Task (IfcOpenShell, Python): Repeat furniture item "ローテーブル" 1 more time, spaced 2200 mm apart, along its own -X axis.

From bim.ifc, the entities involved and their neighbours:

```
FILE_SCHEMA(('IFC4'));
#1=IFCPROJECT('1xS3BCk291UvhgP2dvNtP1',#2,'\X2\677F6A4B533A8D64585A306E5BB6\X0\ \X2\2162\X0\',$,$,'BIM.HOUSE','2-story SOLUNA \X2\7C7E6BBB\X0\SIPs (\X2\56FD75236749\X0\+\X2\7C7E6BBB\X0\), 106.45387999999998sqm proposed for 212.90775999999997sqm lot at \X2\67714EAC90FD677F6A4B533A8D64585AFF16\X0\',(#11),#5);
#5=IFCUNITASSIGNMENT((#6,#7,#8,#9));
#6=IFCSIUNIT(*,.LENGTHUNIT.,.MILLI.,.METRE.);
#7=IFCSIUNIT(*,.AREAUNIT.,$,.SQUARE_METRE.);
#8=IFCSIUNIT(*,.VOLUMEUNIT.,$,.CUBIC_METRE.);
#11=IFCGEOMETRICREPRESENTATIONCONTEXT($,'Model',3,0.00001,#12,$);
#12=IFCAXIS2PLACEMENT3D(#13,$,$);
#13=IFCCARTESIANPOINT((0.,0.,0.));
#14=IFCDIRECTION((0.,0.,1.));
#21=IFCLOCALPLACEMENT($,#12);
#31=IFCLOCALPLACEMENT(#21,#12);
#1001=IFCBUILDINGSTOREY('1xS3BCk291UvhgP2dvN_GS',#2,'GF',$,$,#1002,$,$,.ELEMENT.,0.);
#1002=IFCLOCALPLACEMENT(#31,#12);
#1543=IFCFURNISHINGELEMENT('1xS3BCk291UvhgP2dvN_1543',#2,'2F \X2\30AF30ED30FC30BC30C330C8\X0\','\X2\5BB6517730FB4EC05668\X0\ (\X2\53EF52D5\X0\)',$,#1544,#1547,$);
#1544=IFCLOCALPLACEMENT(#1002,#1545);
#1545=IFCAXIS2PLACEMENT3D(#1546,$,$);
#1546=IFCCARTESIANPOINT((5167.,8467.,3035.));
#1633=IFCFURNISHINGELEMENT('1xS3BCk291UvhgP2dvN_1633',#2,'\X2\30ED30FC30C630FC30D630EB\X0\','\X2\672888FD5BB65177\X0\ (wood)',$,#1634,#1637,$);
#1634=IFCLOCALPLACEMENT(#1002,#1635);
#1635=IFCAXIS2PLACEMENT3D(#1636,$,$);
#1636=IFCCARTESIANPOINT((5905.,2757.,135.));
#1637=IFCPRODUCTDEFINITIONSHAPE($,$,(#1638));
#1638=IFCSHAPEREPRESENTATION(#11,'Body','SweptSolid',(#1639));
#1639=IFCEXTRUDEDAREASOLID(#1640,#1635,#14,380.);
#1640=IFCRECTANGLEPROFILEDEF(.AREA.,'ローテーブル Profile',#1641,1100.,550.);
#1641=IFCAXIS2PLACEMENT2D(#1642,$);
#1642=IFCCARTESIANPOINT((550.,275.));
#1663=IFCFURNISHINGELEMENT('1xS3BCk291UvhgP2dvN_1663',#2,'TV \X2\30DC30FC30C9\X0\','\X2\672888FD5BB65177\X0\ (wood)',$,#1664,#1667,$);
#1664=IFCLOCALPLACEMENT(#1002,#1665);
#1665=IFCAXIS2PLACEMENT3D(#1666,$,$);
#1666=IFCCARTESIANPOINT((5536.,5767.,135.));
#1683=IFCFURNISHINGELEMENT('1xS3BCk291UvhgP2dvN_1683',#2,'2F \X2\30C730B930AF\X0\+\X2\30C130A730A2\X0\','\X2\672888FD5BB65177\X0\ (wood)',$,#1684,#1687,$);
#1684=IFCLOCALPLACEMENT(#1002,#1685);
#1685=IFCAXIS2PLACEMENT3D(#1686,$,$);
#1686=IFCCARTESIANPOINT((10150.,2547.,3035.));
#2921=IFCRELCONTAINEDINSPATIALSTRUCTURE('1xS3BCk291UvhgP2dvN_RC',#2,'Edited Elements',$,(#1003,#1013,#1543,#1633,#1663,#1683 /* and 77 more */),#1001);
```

```python
import ifcopenshell
import ifcopenshell.api.geometry
import ifcopenshell.api.root
import ifcopenshell.util.element
import ifcopenshell.util.placement
import ifcopenshell.util.unit

model = ifcopenshell.open("bim.ifc")
unit_scale = ifcopenshell.util.unit.calculate_unit_scale(model)


def reuse_history(source, copy):
    """copy_class also copies each property set's owner history, people and application; keep the originals."""
    for rel in copy.IsDefinedBy:
        if rel.is_a("IfcRelDefinesByProperties") and (history := rel.RelatingPropertyDefinition.OwnerHistory):
            rel.RelatingPropertyDefinition.OwnerHistory = source.OwnerHistory
            ifcopenshell.util.element.remove_deep2(model, history)


source = model.by_id(1633)
base = ifcopenshell.util.placement.get_local_placement(source.ObjectPlacement)
step = -base[:3, 0] * 2.2 / unit_scale

for i in range(1, 2):
    copy = ifcopenshell.api.root.copy_class(model, product=source)
    copy.Representation = ifcopenshell.util.element.copy_deep(
        model, source.Representation, exclude=["IfcGeometricRepresentationContext", "IfcRepresentationMap"]
    )
    reuse_history(source, copy)
    matrix = base.copy()
    matrix[:3, 3] += i * step
    print("added at", matrix[:3, 3].round(3) + 0.0)
    ifcopenshell.api.geometry.edit_object_placement(model, product=copy, matrix=matrix, is_si=False)

model.write("bim_v2.ifc")
```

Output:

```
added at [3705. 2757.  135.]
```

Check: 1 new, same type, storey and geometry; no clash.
